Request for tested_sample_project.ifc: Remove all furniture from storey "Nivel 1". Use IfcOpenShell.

First a look at what the model holds.

```python
import ifcopenshell
import ifcopenshell.util.element

model = ifcopenshell.open("tested_sample_project.ifc")
print(model.schema)
storey = next(s for s in model.by_type("IfcBuildingStorey") if s.Name == "Nivel 1")
furniture = [e for e in ifcopenshell.util.element.get_decomposition(storey) if e.is_a("IfcFurnishingElement")]
seen = {}
for e in furniture:
    element_type = ifcopenshell.util.element.get_type(e)
    name = element_type.Name if element_type not in (None, e) else None
    seen[name] = seen.get(name, 0) + 1
for name, count in sorted(seen.items(), key=str):
    print(count, "x", name)
```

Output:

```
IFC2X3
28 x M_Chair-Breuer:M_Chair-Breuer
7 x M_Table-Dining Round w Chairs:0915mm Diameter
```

```python
import ifcopenshell
import ifcopenshell.api.root
import ifcopenshell.util.element

model = ifcopenshell.open("tested_sample_project.ifc")

storey = next(s for s in model.by_type("IfcBuildingStorey") if s.Name == "Nivel 1")
furniture = [e for e in ifcopenshell.util.element.get_decomposition(storey) if e.is_a("IfcFurnishingElement")]

for e in furniture:
    ifcopenshell.api.root.remove_product(model, product=e)
print(len(furniture), "removed")

model.write("tested_sample_project_updated.ifc")
```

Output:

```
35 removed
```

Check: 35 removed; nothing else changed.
